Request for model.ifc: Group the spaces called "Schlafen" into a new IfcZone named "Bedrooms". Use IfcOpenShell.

First a look at what the model holds.

```python
import ifcopenshell

model = ifcopenshell.open("model.ifc")
print(model.schema)
seen = {}
for space in model.by_type("IfcSpace"):
    seen[space.LongName] = seen.get(space.LongName, 0) + 1
for name, count in sorted(seen.items(), key=str):
    print(count, "x", name)
print("zones:", [z.Name for z in model.by_type("IfcZone")][:20])
```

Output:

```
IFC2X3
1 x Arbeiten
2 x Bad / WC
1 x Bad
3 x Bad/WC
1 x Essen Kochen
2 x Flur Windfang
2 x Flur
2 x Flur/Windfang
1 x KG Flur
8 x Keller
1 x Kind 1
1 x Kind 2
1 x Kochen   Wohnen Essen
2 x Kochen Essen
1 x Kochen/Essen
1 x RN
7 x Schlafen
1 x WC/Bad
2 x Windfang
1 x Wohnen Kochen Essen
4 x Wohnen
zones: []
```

```python
import ifcopenshell
import ifcopenshell.api.group
import ifcopenshell.api.root

model = ifcopenshell.open("model.ifc")

names = {"Schlafen"}
spaces = [s for s in model.by_type("IfcSpace") if s.LongName in names]

zone = ifcopenshell.api.root.create_entity(model, ifc_class="IfcZone", name="Bedrooms")
ifcopenshell.api.group.assign_group(model, products=spaces, group=zone)
print(len(spaces), "spaces in", zone.Name)

model.write("model_v2.ifc")
```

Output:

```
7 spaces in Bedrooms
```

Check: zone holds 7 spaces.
